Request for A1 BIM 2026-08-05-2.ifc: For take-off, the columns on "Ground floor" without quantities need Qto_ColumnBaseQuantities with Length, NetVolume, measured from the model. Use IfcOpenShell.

First a look at what the model holds.

```python
import ifcopenshell
import ifcopenshell.util.element
import ifcopenshell.util.unit

model = ifcopenshell.open("A1 BIM 2026-08-05-2.ifc")
print(model.schema)
for unit_type in ("LENGTHUNIT", "AREAUNIT", "VOLUMEUNIT"):
    print(unit_type, ifcopenshell.util.unit.calculate_unit_scale(model, unit_type))
storey = next(s for s in model.by_type("IfcBuildingStorey") if s.Name == "Ground floor")
columns = [e for e in ifcopenshell.util.element.get_decomposition(storey) if e.is_a("IfcColumn")]
for e in sorted(columns, key=lambda e: e.id()):
    print(e.id(), e.is_a(), e.Name, list(ifcopenshell.util.element.get_psets(e, qtos_only=True)), sep=" | ")
```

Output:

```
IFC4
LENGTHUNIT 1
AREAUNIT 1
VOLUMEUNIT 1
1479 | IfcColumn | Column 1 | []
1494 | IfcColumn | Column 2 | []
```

```python
import ifcopenshell
import ifcopenshell.api.pset
import ifcopenshell.geom
import ifcopenshell.util.element
import ifcopenshell.util.shape
import ifcopenshell.util.unit

model = ifcopenshell.open("A1 BIM 2026-08-05-2.ifc")
unit_scale = ifcopenshell.util.unit.calculate_unit_scale(model)
volume_scale = ifcopenshell.util.unit.calculate_unit_scale(model, "VOLUMEUNIT")
settings = ifcopenshell.geom.settings()

storey = next(s for s in model.by_type("IfcBuildingStorey") if s.Name == "Ground floor")
columns = [e for e in ifcopenshell.util.element.get_decomposition(storey) if e.is_a("IfcColumn")]

for e in sorted(columns, key=lambda e: e.id()):
    if ifcopenshell.util.element.get_psets(e, qtos_only=True, should_inherit=False):
        continue
    # Geometry comes back in metres, in the element's own axes.
    shape = ifcopenshell.geom.create_shape(settings, e)
    values = {
        "Length": ifcopenshell.util.shape.get_z(shape.geometry) / unit_scale,
        "NetVolume": ifcopenshell.util.shape.get_volume(shape.geometry) / volume_scale,
    }
    qto = ifcopenshell.api.pset.add_qto(model, product=e, name="Qto_ColumnBaseQuantities")
    ifcopenshell.api.pset.edit_qto(model, qto=qto, properties=values)
    print(e.id(), {k: round(v, 3) for k, v in values.items()})

model.write("A1 BIM 2026-08-05-2_rev.ifc")
```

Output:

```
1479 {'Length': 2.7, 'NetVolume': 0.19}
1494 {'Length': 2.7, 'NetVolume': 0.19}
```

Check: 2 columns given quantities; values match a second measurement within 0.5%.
